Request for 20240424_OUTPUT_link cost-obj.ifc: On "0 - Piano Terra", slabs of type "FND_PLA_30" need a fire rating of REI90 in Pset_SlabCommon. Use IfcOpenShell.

First a look at what the model holds.

```python
import ifcopenshell
import ifcopenshell.util.element

model = ifcopenshell.open("20240424_OUTPUT_link cost-obj.ifc")
print(model.schema)
storey = next(s for s in model.by_type("IfcBuildingStorey") if s.Name == "0 - Piano Terra")
slabs = [e for e in ifcopenshell.util.element.get_decomposition(storey) if e.is_a("IfcSlab")]
seen = {}
for e in slabs:
    element_type = ifcopenshell.util.element.get_type(e)
    key = (element_type.Name if element_type != e and element_type else None, ifcopenshell.util.element.get_pset(e, "Pset_SlabCommon", "FireRating"))
    seen[key] = seen.get(key, 0) + 1
for (name, value), count in sorted(seen.items(), key=str):
    print(count, "x", name, "|", value)
```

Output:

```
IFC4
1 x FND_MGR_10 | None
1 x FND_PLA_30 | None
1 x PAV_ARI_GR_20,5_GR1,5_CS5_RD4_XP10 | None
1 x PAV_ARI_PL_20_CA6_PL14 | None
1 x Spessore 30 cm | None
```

```python
import ifcopenshell
import ifcopenshell.api.pset
import ifcopenshell.util.element

model = ifcopenshell.open("20240424_OUTPUT_link cost-obj.ifc")

storey = next(s for s in model.by_type("IfcBuildingStorey") if s.Name == "0 - Piano Terra")
slabs = [e for e in ifcopenshell.util.element.get_decomposition(storey) if e.is_a("IfcSlab")]

count = 0
for e in slabs:
    element_type = ifcopenshell.util.element.get_type(e)
    if element_type in (None, e) or element_type.Name != "FND_PLA_30":
        continue
    # add_pset returns the element's existing set when there is one.
    pset = ifcopenshell.api.pset.add_pset(model, product=e, name="Pset_SlabCommon")
    ifcopenshell.api.pset.edit_pset(model, pset=pset, properties={"FireRating": "REI90"})
    count += 1

print(count, "slabs updated")

model.write("20240424_OUTPUT_link cost-obj_edited.ifc")
```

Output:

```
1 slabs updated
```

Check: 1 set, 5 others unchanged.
